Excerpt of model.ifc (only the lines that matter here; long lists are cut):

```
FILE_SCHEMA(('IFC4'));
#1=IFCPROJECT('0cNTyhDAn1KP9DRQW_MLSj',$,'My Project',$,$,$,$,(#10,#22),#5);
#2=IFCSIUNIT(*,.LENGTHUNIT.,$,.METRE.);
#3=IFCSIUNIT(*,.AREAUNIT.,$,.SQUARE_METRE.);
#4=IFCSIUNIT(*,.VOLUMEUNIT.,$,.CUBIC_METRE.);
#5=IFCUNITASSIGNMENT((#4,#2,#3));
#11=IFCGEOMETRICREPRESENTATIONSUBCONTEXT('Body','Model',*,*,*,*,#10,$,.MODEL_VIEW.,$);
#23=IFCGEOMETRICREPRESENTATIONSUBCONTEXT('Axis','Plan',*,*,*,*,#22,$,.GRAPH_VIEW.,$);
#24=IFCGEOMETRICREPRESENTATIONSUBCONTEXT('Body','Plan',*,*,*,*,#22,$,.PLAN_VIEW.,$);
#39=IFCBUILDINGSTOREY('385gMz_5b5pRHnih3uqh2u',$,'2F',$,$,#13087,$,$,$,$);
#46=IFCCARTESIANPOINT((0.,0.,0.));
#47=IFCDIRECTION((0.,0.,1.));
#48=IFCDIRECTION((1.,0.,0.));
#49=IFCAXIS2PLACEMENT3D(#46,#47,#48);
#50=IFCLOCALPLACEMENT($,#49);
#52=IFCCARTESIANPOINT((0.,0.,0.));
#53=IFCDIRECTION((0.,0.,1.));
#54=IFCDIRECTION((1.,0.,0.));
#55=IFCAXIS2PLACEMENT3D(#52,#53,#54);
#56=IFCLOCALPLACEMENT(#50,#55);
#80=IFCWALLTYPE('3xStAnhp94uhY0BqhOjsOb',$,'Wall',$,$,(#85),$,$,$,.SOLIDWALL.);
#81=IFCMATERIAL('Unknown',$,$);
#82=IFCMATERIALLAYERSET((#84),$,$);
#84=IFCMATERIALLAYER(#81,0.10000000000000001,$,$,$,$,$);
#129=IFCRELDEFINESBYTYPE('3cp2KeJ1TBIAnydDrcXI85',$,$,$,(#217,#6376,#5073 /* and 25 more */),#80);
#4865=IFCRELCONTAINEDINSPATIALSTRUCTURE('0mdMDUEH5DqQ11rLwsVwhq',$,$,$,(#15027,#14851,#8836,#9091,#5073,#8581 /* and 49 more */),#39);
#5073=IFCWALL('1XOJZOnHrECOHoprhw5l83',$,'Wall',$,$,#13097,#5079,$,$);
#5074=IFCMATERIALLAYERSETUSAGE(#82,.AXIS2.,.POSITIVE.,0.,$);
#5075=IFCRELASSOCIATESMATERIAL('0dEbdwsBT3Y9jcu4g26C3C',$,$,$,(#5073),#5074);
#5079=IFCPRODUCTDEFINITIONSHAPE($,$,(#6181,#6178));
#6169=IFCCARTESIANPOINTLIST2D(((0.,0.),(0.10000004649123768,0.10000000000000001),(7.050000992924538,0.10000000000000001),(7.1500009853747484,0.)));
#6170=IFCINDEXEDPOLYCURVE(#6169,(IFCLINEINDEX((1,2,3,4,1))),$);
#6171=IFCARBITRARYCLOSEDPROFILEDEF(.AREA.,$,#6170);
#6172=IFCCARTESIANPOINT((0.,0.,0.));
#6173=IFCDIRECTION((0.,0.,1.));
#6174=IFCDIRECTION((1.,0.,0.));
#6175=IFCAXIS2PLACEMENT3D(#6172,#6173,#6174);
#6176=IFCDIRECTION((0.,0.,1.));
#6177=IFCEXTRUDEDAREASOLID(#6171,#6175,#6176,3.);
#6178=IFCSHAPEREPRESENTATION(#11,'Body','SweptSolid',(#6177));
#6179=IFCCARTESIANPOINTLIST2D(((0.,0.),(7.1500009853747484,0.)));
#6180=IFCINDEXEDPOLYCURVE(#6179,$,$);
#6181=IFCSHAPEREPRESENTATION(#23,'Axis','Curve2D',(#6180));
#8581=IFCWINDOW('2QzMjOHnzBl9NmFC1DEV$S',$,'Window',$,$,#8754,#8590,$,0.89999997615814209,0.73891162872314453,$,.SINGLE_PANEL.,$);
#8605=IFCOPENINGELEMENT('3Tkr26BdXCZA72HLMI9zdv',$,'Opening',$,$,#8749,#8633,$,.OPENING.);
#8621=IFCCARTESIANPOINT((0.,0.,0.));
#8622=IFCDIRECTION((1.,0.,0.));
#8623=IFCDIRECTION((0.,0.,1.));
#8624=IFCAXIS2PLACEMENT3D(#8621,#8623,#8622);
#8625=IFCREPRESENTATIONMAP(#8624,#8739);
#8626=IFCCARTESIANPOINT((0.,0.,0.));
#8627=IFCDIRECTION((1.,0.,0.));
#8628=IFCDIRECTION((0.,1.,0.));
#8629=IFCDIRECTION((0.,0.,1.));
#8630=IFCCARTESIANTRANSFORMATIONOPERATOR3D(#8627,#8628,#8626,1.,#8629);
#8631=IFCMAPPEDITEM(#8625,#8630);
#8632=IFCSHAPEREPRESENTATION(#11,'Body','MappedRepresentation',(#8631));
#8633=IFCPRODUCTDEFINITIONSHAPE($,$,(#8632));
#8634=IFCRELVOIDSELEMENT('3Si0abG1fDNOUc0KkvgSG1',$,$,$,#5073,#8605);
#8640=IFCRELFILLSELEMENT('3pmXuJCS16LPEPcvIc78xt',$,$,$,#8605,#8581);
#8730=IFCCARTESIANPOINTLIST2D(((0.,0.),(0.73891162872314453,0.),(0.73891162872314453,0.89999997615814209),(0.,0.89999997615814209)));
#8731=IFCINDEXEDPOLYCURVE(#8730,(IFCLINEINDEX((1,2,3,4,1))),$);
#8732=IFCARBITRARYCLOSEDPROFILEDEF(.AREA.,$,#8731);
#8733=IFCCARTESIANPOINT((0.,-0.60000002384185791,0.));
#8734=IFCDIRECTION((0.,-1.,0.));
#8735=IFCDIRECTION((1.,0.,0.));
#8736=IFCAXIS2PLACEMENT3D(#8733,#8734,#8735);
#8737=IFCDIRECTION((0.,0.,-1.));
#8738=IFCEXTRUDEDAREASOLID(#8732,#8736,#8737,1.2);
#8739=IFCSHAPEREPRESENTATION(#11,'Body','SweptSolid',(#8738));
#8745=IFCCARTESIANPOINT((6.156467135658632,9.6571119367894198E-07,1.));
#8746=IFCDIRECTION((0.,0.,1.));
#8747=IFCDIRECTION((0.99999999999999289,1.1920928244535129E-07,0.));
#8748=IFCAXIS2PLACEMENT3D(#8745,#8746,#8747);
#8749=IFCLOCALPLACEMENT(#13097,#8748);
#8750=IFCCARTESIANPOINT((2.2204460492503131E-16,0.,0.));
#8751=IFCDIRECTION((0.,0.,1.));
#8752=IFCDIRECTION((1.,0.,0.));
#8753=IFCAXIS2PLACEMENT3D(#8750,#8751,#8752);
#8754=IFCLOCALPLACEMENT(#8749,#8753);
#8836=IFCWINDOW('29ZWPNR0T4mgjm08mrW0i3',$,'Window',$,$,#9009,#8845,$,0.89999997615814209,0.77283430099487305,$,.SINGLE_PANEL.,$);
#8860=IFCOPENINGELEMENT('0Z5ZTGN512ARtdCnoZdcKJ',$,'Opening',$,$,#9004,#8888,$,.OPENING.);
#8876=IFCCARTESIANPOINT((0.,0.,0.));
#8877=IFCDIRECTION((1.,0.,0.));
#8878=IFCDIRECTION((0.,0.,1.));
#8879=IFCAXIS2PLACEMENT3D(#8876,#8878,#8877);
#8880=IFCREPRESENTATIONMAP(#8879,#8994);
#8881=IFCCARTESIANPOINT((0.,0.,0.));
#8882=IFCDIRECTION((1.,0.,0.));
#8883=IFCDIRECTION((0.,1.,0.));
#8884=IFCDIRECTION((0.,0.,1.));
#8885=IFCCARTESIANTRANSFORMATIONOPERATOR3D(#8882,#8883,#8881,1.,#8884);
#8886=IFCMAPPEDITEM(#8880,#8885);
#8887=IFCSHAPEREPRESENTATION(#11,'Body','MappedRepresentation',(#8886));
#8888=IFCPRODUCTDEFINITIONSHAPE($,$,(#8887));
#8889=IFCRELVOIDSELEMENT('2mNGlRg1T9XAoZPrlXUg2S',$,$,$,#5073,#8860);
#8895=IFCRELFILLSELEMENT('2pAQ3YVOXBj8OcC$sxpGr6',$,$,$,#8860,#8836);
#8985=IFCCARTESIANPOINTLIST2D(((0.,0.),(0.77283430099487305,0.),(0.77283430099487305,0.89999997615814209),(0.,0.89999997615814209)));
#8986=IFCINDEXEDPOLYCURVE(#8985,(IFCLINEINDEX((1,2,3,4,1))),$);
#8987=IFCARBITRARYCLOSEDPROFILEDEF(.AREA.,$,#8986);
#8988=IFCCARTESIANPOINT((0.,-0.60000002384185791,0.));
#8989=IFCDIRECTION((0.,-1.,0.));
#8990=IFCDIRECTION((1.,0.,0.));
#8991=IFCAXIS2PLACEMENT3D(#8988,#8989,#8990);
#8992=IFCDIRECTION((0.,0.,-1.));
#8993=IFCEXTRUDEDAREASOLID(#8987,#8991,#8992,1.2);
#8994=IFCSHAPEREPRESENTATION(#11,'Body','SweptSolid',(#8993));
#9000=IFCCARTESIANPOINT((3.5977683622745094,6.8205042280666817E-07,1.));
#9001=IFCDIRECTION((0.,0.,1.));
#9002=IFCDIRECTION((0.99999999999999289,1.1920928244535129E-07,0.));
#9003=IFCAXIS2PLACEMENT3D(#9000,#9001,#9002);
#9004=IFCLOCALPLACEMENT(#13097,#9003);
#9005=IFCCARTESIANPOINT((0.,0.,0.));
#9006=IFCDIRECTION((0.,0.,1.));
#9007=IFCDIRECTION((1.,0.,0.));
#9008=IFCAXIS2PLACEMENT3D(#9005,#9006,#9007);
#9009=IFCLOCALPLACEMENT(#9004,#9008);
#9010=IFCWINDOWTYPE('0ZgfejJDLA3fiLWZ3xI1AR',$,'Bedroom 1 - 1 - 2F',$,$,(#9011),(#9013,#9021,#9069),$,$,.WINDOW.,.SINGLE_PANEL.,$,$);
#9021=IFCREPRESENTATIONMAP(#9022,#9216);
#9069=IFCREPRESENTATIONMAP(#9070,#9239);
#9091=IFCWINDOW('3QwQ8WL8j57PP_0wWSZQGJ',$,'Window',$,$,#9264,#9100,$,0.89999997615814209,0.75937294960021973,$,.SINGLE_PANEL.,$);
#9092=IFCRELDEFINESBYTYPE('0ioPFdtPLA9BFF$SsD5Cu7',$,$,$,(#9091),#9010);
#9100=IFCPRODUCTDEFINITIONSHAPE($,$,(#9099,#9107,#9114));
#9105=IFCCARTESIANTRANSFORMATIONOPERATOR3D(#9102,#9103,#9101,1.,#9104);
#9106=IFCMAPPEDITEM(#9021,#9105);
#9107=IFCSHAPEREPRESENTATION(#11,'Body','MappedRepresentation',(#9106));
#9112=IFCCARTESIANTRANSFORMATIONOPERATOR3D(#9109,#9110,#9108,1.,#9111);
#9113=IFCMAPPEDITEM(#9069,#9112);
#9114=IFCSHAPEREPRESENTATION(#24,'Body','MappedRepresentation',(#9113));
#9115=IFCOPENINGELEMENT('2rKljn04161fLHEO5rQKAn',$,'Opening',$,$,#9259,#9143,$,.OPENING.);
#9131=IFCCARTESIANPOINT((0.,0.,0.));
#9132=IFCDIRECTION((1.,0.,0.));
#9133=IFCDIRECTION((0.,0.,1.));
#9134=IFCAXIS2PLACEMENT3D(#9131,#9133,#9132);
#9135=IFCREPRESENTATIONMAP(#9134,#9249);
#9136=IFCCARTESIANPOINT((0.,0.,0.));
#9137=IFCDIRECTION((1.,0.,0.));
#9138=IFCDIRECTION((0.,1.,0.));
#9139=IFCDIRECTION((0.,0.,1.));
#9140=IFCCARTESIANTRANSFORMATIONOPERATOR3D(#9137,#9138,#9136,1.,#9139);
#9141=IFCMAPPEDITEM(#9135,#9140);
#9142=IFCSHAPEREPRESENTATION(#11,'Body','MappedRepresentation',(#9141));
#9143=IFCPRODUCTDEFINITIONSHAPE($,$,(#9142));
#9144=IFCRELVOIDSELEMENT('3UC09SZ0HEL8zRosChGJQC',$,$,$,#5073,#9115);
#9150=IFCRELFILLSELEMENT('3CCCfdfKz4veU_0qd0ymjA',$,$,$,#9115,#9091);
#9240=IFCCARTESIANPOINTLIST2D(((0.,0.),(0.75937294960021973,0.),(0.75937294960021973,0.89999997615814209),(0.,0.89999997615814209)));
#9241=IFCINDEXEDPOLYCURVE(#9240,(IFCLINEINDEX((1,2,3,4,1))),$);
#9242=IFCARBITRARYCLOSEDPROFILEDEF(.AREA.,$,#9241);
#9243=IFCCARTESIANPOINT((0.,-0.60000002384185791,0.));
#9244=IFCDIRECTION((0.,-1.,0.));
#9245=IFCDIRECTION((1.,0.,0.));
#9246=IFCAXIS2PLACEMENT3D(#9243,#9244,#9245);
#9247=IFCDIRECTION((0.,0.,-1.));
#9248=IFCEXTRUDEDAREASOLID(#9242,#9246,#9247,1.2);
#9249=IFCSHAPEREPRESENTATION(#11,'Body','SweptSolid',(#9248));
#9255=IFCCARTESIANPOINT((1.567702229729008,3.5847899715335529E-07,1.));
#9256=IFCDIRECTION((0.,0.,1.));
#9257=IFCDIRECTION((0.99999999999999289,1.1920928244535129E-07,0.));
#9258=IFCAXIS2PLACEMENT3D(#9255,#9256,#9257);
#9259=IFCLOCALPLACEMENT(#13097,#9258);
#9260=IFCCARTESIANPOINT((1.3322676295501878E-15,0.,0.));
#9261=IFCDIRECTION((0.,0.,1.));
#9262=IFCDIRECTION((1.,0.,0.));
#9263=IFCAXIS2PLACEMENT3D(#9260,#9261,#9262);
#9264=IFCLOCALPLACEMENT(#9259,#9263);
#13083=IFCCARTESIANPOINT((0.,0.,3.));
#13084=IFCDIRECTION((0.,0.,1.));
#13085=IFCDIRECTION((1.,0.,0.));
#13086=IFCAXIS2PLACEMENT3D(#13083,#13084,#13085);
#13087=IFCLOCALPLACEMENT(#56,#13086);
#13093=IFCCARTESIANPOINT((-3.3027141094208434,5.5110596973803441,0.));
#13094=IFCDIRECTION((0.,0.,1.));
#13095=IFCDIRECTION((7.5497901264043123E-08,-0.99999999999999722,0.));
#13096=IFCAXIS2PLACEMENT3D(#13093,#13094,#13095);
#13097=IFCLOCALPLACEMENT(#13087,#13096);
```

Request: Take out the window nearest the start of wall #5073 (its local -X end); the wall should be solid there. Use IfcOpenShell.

```python
import ifcopenshell
import ifcopenshell.api.feature
import ifcopenshell.api.root
import ifcopenshell.geom
import ifcopenshell.util.shape

model = ifcopenshell.open("model.ifc")
settings = ifcopenshell.geom.settings()


def volume(element):
    """Net volume in cubic metres, openings subtracted."""
    shape = ifcopenshell.geom.create_shape(settings, element)
    return ifcopenshell.util.shape.get_volume(shape.geometry)


window = model.by_guid("3QwQ8WL8j57PP_0wWSZQGJ")
opening = window.FillsVoids[0].RelatingOpeningElement
wall = opening.VoidsElements[0].RelatingBuildingElement
before = volume(wall)

ifcopenshell.api.root.remove_product(model, product=window)
ifcopenshell.api.feature.remove_feature(model, feature=opening)

after = volume(wall)

print(f"wall volume {before:.3f} -> {after:.3f} m3")

model.write("model_updated.ifc")
```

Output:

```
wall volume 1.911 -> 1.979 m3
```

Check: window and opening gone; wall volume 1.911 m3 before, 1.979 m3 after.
